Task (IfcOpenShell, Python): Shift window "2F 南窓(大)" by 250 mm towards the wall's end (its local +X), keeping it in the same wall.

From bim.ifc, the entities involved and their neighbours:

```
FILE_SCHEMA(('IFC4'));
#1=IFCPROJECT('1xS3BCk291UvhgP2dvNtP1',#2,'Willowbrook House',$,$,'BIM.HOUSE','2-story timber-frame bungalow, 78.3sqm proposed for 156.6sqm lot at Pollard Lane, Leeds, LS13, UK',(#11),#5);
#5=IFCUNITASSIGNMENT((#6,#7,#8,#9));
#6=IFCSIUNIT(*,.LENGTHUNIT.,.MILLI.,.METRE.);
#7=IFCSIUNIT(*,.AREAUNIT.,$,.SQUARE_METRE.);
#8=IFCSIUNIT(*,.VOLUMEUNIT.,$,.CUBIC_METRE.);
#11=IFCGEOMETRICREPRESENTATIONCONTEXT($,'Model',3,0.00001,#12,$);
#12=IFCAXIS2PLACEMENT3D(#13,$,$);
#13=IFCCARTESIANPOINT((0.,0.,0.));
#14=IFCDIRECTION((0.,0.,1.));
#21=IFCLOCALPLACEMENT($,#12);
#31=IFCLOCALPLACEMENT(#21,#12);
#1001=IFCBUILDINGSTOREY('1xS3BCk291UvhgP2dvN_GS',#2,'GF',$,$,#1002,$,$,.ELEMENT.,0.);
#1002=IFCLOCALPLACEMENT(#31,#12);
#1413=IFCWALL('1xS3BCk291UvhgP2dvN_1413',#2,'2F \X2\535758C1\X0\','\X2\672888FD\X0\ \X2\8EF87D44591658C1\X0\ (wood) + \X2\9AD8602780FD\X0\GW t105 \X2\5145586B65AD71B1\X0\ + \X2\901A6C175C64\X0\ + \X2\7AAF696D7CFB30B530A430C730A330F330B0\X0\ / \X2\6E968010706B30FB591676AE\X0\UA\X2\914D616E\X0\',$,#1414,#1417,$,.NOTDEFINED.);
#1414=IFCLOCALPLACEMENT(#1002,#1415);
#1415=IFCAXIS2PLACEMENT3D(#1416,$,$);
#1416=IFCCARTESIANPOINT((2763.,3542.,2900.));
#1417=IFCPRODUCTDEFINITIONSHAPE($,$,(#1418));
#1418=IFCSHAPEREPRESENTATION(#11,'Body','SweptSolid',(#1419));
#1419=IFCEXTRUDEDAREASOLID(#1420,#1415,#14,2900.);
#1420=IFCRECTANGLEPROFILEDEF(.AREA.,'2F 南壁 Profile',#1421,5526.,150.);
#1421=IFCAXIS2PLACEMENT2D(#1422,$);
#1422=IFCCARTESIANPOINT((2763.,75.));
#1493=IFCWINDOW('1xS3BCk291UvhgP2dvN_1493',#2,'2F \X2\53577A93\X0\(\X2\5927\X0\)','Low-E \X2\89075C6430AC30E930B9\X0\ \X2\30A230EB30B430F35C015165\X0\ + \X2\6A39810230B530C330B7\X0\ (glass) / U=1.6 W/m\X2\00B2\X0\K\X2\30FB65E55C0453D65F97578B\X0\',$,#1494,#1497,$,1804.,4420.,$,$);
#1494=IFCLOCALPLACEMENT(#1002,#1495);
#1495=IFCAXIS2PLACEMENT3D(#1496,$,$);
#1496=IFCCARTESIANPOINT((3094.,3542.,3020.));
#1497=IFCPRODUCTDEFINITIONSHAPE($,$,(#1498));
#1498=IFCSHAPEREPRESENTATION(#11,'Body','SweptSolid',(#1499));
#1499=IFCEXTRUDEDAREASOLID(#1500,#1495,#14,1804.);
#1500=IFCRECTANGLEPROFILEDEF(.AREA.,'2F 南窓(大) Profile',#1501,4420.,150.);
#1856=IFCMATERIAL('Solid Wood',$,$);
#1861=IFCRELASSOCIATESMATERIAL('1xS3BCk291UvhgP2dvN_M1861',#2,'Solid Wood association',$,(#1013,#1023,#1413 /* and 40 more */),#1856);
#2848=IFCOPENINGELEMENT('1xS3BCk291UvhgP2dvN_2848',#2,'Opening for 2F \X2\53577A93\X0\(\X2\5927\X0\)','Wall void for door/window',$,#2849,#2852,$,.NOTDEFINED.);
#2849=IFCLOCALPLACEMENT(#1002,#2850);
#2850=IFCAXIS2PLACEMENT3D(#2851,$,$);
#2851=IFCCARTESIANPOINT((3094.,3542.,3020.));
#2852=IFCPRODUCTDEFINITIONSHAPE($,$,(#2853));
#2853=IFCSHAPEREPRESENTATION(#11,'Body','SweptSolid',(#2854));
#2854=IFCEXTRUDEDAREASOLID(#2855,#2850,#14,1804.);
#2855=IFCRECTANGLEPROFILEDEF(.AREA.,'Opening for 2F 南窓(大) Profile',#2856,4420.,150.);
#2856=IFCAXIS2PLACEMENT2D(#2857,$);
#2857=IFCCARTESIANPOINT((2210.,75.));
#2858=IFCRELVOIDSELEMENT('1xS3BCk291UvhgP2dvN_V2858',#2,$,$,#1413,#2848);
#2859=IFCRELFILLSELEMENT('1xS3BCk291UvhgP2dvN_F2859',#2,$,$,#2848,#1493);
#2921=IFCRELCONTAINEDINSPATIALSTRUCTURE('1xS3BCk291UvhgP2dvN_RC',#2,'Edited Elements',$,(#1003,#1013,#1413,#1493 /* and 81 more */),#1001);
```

```python
import ifcopenshell
import ifcopenshell.api.geometry
import ifcopenshell.util.placement
import ifcopenshell.util.unit

model = ifcopenshell.open("bim.ifc")
unit_scale = ifcopenshell.util.unit.calculate_unit_scale(model)

window = model.by_guid("1xS3BCk291UvhgP2dvN_1493")
opening = window.FillsVoids[0].RelatingOpeningElement
wall = opening.VoidsElements[0].RelatingBuildingElement

wall_matrix = ifcopenshell.util.placement.get_local_placement(wall.ObjectPlacement)
shift = wall_matrix[:3, 0] * 0.25 / unit_scale
before = ifcopenshell.util.placement.get_local_placement(window.ObjectPlacement)[:3, 3].copy()

# The window is not placed relative to its opening, so move both.
for product in (opening, window):
    matrix = ifcopenshell.util.placement.get_local_placement(product.ObjectPlacement)
    matrix[:3, 3] += shift
    ifcopenshell.api.geometry.edit_object_placement(model, product=product, matrix=matrix, is_si=False)

after = ifcopenshell.util.placement.get_local_placement(window.ObjectPlacement)[:3, 3]
print("window moved by", (after - before).round(3) + 0.0)

model.write("bim_rev.ifc")
```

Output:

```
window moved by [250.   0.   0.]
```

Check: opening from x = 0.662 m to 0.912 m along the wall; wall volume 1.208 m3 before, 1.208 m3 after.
